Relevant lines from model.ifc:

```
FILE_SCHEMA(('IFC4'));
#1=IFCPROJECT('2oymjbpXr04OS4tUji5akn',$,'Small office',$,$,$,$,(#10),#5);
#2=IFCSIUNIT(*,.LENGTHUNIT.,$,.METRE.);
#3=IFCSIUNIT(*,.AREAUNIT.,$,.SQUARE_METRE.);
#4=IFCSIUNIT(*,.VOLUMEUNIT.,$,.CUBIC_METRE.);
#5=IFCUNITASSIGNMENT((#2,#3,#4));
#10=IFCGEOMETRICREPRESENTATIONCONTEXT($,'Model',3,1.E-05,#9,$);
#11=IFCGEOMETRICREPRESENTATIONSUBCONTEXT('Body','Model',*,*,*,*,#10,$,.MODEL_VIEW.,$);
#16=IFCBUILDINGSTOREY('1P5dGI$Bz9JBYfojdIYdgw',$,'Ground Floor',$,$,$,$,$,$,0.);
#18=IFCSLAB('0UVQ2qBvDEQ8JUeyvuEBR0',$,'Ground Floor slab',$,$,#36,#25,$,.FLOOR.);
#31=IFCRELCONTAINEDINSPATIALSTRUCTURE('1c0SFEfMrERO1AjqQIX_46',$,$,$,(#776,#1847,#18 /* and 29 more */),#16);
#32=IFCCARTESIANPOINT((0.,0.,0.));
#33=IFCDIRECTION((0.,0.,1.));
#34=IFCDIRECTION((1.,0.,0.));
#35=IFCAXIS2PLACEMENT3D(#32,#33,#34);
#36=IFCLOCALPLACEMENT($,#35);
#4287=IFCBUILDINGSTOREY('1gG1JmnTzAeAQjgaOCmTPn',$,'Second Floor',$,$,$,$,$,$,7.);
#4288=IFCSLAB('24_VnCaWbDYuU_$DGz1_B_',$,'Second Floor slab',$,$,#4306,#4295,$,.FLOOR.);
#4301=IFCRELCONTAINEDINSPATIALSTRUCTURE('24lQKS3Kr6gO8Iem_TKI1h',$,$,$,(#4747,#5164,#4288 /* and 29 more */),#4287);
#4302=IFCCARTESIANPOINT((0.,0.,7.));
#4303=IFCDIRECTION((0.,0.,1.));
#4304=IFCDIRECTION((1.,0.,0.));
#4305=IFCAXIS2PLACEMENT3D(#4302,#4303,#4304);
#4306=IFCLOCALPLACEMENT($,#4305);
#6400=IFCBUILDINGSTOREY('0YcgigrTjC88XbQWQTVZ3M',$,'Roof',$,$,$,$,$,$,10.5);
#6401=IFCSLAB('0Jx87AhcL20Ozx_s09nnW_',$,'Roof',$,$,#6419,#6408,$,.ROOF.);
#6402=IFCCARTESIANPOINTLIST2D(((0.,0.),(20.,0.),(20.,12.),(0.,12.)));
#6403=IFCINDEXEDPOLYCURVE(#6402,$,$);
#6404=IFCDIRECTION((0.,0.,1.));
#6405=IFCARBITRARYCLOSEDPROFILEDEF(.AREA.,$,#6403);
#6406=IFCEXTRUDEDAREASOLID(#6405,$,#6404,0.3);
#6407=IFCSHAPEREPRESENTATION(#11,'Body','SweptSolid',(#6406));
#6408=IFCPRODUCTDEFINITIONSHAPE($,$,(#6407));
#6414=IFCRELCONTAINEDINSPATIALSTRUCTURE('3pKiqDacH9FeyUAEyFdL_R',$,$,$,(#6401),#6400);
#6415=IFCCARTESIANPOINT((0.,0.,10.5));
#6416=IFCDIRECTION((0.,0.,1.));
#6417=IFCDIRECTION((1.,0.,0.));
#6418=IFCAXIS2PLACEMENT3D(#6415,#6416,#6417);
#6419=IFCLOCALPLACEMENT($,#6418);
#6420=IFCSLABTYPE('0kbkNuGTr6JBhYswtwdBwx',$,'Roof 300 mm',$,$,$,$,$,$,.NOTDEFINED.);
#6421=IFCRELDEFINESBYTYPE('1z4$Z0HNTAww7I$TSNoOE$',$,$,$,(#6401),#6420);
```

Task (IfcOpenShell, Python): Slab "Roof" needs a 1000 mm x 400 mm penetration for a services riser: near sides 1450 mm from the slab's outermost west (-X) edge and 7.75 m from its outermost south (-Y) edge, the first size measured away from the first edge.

```python
import numpy as np
import ifcopenshell
import ifcopenshell.api.feature
import ifcopenshell.api.geometry
import ifcopenshell.api.root
import ifcopenshell.geom
import ifcopenshell.util.placement
import ifcopenshell.util.representation
import ifcopenshell.util.shape
import ifcopenshell.util.unit

model = ifcopenshell.open("model.ifc")
unit_scale = ifcopenshell.util.unit.calculate_unit_scale(model)
settings = ifcopenshell.geom.settings()


def volume(element):
    """Net volume in cubic metres, openings subtracted."""
    shape = ifcopenshell.geom.create_shape(settings, element)
    return ifcopenshell.util.shape.get_volume(shape.geometry)


slab = model.by_id(6401)
before = volume(slab)

# Extent in the slab's own axes, in metres. The edges named are its -X and -Y sides.
slab_shape = ifcopenshell.geom.create_shape(settings, slab)
vertices = ifcopenshell.util.shape.get_vertices(slab_shape.geometry)
x_min, y_min, bottom = vertices.min(axis=0)
top = vertices[:, 2].max()

opening = ifcopenshell.api.root.create_entity(model, ifc_class="IfcOpeningElement", name="Services riser opening", predefined_type="OPENING")
context = ifcopenshell.util.representation.get_context(model, "Model", "Body", "MODEL_VIEW")
width, depth = 1, 0.4
outline = [(0.0, 0.0), (width, 0.0), (width, depth), (0.0, depth), (0.0, 0.0)]
# Overshoot both faces by 50 mm so the cut is clean.
shape = ifcopenshell.api.geometry.add_slab_representation(
    model, context=context, depth=top - bottom + 0.1, polyline=outline
)
ifcopenshell.api.geometry.assign_representation(model, product=opening, representation=shape)

matrix = ifcopenshell.util.placement.get_local_placement(slab.ObjectPlacement)
matrix[:, 3] = matrix @ np.append(np.array([x_min + 1.45, y_min + 7.75, bottom - 0.05]) / unit_scale, 1.0)
ifcopenshell.api.geometry.edit_object_placement(model, product=opening, matrix=matrix, is_si=False)
ifcopenshell.api.feature.add_feature(model, feature=opening, element=slab)

after = volume(slab)

print(f"slab volume {before:.3f} -> {after:.3f} m3")

model.write("model_v2.ifc")
```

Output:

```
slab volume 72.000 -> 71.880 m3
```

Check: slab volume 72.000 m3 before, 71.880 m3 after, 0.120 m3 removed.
